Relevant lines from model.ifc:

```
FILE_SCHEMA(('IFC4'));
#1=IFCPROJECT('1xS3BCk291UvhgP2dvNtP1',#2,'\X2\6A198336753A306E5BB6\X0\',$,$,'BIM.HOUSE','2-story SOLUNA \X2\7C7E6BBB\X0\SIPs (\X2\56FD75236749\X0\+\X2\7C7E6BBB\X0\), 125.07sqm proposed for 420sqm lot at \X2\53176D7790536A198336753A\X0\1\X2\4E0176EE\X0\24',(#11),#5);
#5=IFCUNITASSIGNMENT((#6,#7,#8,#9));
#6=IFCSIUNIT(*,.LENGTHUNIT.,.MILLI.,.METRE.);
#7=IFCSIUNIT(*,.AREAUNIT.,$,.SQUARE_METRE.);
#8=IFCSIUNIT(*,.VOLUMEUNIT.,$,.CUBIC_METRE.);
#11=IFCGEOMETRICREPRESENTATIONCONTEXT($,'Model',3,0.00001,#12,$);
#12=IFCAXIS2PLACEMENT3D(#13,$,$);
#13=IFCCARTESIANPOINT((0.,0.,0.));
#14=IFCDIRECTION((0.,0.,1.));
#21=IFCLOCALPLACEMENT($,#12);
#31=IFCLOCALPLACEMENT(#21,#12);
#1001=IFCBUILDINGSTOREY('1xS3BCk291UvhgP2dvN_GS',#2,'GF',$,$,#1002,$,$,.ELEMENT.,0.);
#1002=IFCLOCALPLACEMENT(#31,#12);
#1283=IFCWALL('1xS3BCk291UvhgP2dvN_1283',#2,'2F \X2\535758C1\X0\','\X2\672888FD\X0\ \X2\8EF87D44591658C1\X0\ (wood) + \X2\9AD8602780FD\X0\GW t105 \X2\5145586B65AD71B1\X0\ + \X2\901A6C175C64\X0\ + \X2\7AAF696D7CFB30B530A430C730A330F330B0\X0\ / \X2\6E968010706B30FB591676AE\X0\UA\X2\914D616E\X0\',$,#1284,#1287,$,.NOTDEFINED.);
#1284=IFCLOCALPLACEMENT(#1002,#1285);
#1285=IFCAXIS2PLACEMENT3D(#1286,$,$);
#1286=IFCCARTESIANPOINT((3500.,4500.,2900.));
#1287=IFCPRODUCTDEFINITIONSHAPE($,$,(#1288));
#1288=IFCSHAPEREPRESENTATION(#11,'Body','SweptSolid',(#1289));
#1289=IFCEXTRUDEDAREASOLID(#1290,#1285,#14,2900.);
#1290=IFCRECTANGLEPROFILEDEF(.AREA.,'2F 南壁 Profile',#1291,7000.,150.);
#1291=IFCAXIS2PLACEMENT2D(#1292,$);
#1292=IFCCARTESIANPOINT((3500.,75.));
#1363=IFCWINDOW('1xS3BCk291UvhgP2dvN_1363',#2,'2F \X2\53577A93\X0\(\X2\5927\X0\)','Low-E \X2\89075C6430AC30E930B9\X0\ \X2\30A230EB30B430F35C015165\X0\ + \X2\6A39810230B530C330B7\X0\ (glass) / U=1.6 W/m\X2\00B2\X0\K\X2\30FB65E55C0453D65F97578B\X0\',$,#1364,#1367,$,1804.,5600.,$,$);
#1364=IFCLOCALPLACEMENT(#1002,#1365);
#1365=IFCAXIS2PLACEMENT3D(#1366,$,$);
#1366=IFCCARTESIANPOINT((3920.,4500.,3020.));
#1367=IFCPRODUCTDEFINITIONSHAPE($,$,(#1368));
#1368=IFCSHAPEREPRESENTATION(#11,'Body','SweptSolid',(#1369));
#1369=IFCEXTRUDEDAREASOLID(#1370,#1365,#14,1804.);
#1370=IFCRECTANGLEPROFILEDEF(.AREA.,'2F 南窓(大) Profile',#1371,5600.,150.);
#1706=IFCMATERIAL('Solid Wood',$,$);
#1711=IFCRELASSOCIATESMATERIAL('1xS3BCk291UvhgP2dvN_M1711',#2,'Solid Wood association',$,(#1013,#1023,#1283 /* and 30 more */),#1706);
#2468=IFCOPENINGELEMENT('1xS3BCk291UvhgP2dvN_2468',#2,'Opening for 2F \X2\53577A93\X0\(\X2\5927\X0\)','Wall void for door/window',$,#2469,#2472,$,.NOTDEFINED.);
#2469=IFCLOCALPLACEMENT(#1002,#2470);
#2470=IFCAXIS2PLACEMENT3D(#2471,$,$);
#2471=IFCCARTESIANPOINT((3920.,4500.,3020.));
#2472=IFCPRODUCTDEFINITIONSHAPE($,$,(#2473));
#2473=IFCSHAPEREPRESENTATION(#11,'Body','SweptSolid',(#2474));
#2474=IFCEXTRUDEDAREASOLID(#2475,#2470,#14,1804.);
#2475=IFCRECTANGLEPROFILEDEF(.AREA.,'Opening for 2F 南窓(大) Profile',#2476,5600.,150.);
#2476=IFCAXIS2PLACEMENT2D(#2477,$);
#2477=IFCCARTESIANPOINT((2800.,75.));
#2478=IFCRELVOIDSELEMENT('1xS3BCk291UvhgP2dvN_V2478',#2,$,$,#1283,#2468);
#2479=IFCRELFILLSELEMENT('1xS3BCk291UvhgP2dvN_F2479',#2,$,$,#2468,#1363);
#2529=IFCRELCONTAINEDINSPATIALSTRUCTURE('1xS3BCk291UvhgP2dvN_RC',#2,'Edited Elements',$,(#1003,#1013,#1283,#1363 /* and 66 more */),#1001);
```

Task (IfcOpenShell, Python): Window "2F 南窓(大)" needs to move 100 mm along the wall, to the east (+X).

```python
import ifcopenshell
import ifcopenshell.api.geometry
import ifcopenshell.util.placement
import ifcopenshell.util.unit

model = ifcopenshell.open("model.ifc")
unit_scale = ifcopenshell.util.unit.calculate_unit_scale(model)

window = model.by_guid("1xS3BCk291UvhgP2dvN_1363")
opening = window.FillsVoids[0].RelatingOpeningElement
wall = opening.VoidsElements[0].RelatingBuildingElement

wall_matrix = ifcopenshell.util.placement.get_local_placement(wall.ObjectPlacement)
shift = wall_matrix[:3, 0] * 0.1 / unit_scale
before = ifcopenshell.util.placement.get_local_placement(window.ObjectPlacement)[:3, 3].copy()

# The window is not placed relative to its opening, so move both.
for product in (opening, window):
    matrix = ifcopenshell.util.placement.get_local_placement(product.ObjectPlacement)
    matrix[:3, 3] += shift
    ifcopenshell.api.geometry.edit_object_placement(model, product=product, matrix=matrix, is_si=False)

after = ifcopenshell.util.placement.get_local_placement(window.ObjectPlacement)[:3, 3]
print("window moved by", (after - before).round(3) + 0.0)

model.write("model_v2.ifc")
```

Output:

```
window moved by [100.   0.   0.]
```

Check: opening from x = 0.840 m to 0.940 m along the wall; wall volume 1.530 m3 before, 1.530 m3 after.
